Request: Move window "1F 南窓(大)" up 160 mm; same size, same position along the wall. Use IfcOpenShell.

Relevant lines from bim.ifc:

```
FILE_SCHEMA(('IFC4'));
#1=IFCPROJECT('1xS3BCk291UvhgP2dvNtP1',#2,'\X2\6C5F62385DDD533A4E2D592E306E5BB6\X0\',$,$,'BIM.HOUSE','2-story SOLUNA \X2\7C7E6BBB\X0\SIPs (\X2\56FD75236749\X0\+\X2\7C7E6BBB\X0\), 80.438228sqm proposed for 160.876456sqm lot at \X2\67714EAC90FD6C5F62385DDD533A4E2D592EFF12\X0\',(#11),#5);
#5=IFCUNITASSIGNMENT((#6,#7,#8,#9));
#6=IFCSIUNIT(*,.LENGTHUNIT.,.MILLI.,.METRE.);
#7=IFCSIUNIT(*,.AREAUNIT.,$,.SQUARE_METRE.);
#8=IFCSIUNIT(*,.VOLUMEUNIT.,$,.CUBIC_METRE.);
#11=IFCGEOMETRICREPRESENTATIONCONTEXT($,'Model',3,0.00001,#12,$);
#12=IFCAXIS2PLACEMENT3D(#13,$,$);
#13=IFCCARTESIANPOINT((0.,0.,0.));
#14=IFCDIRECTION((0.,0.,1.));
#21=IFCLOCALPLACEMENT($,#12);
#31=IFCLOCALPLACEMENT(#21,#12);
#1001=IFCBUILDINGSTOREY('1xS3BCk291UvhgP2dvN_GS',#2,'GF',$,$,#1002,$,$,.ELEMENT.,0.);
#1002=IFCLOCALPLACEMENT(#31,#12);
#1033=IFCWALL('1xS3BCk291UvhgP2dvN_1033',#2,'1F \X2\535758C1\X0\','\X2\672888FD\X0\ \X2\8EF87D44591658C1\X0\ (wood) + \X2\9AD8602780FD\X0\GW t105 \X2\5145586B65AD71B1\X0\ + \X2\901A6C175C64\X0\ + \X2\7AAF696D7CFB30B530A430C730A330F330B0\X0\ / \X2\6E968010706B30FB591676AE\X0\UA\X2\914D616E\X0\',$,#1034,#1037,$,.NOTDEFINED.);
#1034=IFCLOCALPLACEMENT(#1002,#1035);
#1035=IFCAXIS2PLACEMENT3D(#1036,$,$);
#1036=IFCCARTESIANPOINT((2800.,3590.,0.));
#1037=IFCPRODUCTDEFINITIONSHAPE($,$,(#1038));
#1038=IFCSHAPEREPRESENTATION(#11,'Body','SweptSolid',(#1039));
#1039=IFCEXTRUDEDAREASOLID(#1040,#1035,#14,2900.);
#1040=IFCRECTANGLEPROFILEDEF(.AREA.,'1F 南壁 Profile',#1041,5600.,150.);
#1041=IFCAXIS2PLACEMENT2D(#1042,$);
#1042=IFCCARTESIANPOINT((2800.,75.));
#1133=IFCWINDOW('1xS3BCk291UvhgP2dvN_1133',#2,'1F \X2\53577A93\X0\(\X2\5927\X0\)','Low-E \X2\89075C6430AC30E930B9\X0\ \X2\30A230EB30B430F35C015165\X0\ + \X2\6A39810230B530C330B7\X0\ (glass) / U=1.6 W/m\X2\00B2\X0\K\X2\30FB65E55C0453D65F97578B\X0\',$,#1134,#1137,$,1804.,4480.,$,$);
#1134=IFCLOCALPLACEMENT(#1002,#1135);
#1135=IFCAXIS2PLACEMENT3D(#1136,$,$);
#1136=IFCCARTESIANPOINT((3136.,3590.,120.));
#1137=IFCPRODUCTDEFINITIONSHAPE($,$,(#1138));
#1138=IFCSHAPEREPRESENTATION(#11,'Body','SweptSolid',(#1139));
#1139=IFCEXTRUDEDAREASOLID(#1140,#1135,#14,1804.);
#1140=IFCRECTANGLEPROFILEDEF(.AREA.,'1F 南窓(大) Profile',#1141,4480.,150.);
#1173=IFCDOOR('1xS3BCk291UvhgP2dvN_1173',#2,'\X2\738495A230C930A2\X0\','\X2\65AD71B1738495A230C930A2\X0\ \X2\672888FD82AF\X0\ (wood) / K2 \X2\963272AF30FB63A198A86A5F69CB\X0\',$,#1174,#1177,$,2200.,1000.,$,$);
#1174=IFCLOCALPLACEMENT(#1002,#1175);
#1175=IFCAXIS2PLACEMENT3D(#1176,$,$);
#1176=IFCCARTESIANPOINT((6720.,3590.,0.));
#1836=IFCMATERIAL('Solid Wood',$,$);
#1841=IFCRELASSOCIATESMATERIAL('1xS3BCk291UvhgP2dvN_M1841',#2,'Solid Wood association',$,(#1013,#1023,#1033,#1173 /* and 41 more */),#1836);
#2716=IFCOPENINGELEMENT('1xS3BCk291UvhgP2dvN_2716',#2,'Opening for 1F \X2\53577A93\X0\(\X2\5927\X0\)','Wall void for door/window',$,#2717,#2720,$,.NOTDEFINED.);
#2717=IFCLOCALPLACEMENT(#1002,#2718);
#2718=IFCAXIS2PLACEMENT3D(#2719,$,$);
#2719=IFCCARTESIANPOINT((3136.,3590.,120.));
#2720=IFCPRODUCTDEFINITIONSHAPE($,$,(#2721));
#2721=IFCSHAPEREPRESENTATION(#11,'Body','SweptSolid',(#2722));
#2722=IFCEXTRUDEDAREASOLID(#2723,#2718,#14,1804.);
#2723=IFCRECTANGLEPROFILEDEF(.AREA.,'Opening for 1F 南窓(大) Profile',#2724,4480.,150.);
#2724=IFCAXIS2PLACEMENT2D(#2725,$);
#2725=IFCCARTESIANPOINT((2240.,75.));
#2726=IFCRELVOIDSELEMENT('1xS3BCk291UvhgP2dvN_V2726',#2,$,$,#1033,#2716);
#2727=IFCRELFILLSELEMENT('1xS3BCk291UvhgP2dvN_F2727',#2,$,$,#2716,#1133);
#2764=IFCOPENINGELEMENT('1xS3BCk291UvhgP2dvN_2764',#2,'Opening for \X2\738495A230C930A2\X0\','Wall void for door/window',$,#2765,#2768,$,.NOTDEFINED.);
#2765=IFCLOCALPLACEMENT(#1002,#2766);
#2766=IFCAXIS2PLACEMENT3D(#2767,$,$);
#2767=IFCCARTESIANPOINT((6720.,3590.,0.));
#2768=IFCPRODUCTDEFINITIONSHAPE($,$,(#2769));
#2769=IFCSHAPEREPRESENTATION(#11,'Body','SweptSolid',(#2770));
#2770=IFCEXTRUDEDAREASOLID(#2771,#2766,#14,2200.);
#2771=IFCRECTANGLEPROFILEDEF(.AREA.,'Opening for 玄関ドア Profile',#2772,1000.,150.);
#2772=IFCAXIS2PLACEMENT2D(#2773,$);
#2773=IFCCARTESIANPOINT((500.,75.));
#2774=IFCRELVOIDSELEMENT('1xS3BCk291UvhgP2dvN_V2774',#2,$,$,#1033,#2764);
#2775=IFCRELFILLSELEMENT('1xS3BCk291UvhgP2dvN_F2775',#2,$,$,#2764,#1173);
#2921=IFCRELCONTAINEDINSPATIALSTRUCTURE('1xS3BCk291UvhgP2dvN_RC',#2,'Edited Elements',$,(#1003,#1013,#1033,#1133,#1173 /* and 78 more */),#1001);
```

```python
import numpy as np
import ifcopenshell
import ifcopenshell.api.geometry
import ifcopenshell.util.placement
import ifcopenshell.util.unit

model = ifcopenshell.open("bim.ifc")
unit_scale = ifcopenshell.util.unit.calculate_unit_scale(model)

window = model.by_id(1133)
opening = window.FillsVoids[0].RelatingOpeningElement
dz = 0.16 / unit_scale

shift = np.array([0.0, 0.0, dz])
# The window is not placed relative to its opening, so move both.
for product in (opening, window):
    matrix = ifcopenshell.util.placement.get_local_placement(product.ObjectPlacement)
    matrix[:3, 3] += shift
    ifcopenshell.api.geometry.edit_object_placement(model, product=product, matrix=matrix, is_si=False)

print(f"moved by {dz * unit_scale:+.3f} m")

model.write("bim-out.ifc")
```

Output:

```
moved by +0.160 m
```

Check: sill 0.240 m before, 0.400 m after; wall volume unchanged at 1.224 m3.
